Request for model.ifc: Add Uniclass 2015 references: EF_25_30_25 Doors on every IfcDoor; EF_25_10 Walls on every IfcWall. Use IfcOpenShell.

First a look at what the model holds.

```python
import ifcopenshell

model = ifcopenshell.open("model.ifc")
print(model.schema)
print("classifications:", [c.Name for c in model.by_type("IfcClassification")])
for ifc_class in ("IfcDoor", "IfcRoof", "IfcStair", "IfcWall", "IfcWindow"):
    print(ifc_class, len(model.by_type(ifc_class)))
```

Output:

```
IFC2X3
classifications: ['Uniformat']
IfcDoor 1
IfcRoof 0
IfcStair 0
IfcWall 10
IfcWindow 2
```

```python
import ifcopenshell
import ifcopenshell.api.classification

model = ifcopenshell.open("model.ifc")

# IFC2X3 requires Source and Edition and has no link from the project to the system.
system = model.create_entity("IfcClassification", Source="NBS", Edition="2015", Name="Uniclass 2015")

codes = {
    "IfcDoor": ("EF_25_30_25", "Doors"),
    "IfcWall": ("EF_25_10", "Walls"),
}
for ifc_class, (code, name) in codes.items():
    products = model.by_type(ifc_class)
    ifcopenshell.api.classification.add_reference(
        model, products=products, classification=system, identification=code, name=name
    )
    print(code, len(products))

model.write("model_v2.ifc")
```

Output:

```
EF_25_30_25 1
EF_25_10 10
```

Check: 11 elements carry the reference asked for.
